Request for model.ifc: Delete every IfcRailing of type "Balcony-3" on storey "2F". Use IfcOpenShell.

First a look at what the model holds.

```python
import ifcopenshell
import ifcopenshell.util.element

model = ifcopenshell.open("model.ifc")
print(model.schema)
storey = next(s for s in model.by_type("IfcBuildingStorey") if s.Name == "2F")
railings = [e for e in ifcopenshell.util.element.get_decomposition(storey) if e.is_a("IfcRailing")]
seen = {}
for e in railings:
    element_type = ifcopenshell.util.element.get_type(e)
    name = element_type.Name if element_type not in (None, e) else None
    seen[name] = seen.get(name, 0) + 1
for name, count in sorted(seen.items(), key=str):
    print(count, "x", name)
```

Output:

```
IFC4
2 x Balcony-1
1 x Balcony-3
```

```python
import ifcopenshell
import ifcopenshell.api.root
import ifcopenshell.util.element

model = ifcopenshell.open("model.ifc")

storey = next(s for s in model.by_type("IfcBuildingStorey") if s.Name == "2F")
railings = [e for e in ifcopenshell.util.element.get_decomposition(storey) if e.is_a("IfcRailing")]
targets = [e for e in railings if (t := ifcopenshell.util.element.get_type(e)) not in (None, e) and t.Name == "Balcony-3"]

for e in targets:
    ifcopenshell.api.root.remove_product(model, product=e)
print(len(targets), "removed")

model.write("model_updated.ifc")
```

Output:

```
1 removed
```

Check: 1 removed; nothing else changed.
